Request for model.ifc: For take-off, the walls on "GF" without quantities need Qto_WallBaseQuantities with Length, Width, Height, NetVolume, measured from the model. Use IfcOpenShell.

First a look at what the model holds.

```python
import ifcopenshell
import ifcopenshell.util.element
import ifcopenshell.util.unit

model = ifcopenshell.open("model.ifc")
print(model.schema)
for unit_type in ("LENGTHUNIT", "AREAUNIT", "VOLUMEUNIT"):
    print(unit_type, ifcopenshell.util.unit.calculate_unit_scale(model, unit_type))
storey = next(s for s in model.by_type("IfcBuildingStorey") if s.Name == "GF")
walls = [e for e in ifcopenshell.util.element.get_decomposition(storey) if e.is_a("IfcWall")]
for e in sorted(walls, key=lambda e: e.id()):
    print(e.id(), e.is_a(), e.Name, list(ifcopenshell.util.element.get_psets(e, qtos_only=True)), sep=" | ")
```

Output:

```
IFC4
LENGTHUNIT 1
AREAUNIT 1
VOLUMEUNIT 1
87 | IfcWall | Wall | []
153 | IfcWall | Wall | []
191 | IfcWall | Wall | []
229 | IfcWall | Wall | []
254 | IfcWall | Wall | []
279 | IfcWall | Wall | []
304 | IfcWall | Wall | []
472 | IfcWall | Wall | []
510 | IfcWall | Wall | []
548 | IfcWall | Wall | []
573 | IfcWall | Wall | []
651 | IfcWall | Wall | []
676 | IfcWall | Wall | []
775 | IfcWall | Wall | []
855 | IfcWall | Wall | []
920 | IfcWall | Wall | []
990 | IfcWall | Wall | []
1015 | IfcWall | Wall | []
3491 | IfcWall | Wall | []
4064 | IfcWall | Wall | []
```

```python
import ifcopenshell
import ifcopenshell.api.pset
import ifcopenshell.geom
import ifcopenshell.util.element
import ifcopenshell.util.shape
import ifcopenshell.util.unit

model = ifcopenshell.open("model.ifc")
unit_scale = ifcopenshell.util.unit.calculate_unit_scale(model)
volume_scale = ifcopenshell.util.unit.calculate_unit_scale(model, "VOLUMEUNIT")
settings = ifcopenshell.geom.settings()

storey = next(s for s in model.by_type("IfcBuildingStorey") if s.Name == "GF")
walls = [e for e in ifcopenshell.util.element.get_decomposition(storey) if e.is_a("IfcWall")]

for e in sorted(walls, key=lambda e: e.id()):
    if ifcopenshell.util.element.get_psets(e, qtos_only=True, should_inherit=False):
        continue
    # Geometry comes back in metres, in the element's own axes.
    shape = ifcopenshell.geom.create_shape(settings, e)
    values = {
        "Length": ifcopenshell.util.shape.get_x(shape.geometry) / unit_scale,
        "Width": ifcopenshell.util.shape.get_y(shape.geometry) / unit_scale,
        "Height": ifcopenshell.util.shape.get_z(shape.geometry) / unit_scale,
        "NetVolume": ifcopenshell.util.shape.get_volume(shape.geometry) / volume_scale,
    }
    qto = ifcopenshell.api.pset.add_qto(model, product=e, name="Qto_WallBaseQuantities")
    ifcopenshell.api.pset.edit_qto(model, qto=qto, properties=values)
    print(e.id(), {k: round(v, 3) for k, v in values.items()})

model.write("model_rev.ifc")
```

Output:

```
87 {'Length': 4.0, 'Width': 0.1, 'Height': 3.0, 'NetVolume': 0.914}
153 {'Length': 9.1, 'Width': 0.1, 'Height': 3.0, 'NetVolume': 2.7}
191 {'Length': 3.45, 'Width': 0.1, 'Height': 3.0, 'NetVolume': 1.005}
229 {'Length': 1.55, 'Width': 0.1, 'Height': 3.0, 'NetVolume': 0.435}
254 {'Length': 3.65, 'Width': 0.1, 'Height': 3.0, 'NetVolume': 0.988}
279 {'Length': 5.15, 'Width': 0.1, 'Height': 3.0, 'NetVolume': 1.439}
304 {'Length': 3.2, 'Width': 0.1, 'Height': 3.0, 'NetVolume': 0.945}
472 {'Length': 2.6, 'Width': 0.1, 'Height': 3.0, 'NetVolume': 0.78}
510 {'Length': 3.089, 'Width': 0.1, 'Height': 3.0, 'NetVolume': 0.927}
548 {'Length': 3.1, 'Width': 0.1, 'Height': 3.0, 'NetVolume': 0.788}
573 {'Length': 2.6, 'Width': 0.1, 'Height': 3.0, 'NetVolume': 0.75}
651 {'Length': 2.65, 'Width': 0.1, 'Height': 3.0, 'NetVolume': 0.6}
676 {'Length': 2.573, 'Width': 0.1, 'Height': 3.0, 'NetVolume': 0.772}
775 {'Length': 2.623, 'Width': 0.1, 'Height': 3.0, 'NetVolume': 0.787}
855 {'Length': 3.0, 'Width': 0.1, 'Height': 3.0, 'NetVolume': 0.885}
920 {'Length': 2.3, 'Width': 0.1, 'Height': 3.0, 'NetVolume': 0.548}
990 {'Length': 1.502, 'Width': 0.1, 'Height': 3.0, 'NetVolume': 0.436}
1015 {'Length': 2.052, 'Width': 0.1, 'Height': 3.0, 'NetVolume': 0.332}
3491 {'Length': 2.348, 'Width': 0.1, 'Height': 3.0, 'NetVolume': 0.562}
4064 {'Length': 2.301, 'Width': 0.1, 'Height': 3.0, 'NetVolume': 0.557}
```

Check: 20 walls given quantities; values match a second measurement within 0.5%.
